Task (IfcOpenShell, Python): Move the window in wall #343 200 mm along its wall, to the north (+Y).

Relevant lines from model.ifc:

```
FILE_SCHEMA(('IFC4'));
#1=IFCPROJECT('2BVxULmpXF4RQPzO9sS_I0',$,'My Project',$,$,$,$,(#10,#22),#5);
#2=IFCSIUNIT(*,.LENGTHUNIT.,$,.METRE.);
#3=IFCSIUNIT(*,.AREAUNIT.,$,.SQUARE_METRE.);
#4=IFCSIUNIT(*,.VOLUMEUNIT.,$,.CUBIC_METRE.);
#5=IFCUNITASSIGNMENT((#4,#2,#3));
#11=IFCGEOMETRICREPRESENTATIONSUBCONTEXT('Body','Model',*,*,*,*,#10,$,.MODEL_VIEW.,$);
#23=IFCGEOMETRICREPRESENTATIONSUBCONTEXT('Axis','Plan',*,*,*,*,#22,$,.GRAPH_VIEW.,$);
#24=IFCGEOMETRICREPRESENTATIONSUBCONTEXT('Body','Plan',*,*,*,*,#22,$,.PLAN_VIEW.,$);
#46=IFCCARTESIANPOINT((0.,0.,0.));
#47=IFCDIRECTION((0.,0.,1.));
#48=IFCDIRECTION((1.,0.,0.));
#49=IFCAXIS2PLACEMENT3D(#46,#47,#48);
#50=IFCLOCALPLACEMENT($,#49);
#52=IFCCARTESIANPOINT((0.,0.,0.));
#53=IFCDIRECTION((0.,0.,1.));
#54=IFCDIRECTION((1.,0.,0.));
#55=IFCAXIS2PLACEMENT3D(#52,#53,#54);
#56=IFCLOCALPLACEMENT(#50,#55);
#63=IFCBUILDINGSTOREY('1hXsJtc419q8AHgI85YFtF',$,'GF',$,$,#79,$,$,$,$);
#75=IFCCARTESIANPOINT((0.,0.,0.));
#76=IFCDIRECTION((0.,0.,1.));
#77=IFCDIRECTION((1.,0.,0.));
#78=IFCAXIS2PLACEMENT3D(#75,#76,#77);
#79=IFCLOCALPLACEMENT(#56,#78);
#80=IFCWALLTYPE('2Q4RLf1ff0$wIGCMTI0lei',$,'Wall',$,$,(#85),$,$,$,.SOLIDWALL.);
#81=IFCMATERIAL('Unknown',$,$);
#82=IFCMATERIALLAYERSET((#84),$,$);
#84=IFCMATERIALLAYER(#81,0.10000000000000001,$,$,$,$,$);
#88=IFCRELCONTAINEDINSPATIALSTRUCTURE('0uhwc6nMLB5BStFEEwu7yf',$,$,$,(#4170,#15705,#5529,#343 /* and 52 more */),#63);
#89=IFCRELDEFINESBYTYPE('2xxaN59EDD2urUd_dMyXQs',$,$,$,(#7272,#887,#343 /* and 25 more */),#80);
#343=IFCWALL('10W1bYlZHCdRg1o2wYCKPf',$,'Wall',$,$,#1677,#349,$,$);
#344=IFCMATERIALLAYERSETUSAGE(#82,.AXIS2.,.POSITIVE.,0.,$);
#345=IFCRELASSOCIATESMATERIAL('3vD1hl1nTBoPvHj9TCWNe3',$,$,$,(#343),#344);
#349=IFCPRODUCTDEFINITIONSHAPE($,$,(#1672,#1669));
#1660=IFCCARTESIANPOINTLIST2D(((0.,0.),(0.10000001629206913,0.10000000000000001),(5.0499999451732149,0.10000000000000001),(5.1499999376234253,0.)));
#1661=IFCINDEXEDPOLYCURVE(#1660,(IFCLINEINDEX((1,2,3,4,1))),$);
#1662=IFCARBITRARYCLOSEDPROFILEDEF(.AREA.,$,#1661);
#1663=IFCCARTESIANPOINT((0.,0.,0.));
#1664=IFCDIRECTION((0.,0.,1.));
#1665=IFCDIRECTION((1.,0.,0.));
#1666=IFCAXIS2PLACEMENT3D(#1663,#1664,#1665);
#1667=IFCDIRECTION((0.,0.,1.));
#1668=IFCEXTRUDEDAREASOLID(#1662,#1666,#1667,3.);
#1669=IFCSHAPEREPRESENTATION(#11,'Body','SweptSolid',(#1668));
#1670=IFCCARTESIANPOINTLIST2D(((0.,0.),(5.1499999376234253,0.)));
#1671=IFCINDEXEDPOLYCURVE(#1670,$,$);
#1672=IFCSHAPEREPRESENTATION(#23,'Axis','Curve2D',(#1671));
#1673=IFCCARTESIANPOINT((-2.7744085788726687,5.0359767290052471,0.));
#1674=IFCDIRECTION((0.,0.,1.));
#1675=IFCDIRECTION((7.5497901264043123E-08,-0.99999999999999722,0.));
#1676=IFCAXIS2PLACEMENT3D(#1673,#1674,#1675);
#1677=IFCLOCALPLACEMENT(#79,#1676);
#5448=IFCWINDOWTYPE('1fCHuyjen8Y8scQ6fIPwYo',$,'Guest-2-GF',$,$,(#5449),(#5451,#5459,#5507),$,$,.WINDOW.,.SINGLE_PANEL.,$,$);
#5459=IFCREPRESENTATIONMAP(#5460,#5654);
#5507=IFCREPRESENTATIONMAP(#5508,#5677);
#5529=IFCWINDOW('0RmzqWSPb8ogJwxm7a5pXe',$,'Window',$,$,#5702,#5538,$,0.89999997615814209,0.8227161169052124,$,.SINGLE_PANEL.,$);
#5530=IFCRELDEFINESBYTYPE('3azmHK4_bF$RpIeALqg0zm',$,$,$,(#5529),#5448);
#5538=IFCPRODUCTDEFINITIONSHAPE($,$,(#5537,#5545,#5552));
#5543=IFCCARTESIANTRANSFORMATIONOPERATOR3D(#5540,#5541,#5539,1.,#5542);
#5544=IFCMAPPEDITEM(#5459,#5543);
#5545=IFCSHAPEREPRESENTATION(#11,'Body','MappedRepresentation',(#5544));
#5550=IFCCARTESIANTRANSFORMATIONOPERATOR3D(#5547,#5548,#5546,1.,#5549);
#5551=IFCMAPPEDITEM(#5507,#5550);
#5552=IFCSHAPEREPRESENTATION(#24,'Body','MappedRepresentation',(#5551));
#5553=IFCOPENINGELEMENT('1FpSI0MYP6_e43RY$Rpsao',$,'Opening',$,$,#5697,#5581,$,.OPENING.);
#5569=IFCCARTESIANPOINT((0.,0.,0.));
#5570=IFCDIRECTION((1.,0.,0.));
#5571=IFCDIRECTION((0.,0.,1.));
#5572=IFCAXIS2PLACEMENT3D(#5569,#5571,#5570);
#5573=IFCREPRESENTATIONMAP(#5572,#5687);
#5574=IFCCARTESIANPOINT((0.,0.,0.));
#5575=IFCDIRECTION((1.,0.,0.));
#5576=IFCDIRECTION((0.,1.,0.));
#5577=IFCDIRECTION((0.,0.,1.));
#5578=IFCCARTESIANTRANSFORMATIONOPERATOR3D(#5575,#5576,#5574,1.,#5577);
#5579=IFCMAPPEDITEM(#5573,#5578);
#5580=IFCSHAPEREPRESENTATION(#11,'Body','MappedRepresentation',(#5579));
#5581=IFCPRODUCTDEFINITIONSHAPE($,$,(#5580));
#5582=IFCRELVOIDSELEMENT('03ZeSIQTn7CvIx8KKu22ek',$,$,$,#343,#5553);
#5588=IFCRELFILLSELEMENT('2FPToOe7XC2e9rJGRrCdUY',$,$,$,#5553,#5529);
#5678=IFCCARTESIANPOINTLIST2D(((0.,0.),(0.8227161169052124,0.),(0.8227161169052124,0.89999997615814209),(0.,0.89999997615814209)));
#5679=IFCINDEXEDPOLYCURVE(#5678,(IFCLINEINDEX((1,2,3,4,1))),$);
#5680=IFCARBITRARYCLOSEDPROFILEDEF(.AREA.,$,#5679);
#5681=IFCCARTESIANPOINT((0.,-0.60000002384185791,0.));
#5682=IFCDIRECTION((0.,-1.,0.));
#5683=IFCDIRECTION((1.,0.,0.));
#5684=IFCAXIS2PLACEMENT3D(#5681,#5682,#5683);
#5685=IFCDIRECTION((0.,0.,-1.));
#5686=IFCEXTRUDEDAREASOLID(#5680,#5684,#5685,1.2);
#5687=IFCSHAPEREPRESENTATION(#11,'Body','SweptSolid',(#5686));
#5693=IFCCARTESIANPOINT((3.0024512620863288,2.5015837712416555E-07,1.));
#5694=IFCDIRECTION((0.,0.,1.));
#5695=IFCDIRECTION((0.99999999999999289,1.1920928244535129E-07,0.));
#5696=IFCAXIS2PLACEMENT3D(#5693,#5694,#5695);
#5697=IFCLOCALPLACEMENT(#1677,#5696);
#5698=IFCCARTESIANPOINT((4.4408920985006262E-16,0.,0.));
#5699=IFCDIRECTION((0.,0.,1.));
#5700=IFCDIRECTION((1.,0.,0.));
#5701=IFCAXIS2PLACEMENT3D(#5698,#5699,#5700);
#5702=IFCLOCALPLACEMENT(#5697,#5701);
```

```python
import ifcopenshell
import ifcopenshell.api.geometry
import ifcopenshell.util.placement
import ifcopenshell.util.unit

model = ifcopenshell.open("model.ifc")
unit_scale = ifcopenshell.util.unit.calculate_unit_scale(model)

window = model.by_id(5529)
opening = window.FillsVoids[0].RelatingOpeningElement
wall = opening.VoidsElements[0].RelatingBuildingElement

wall_matrix = ifcopenshell.util.placement.get_local_placement(wall.ObjectPlacement)
shift = wall_matrix[:3, 0] * -0.2 / unit_scale
before = ifcopenshell.util.placement.get_local_placement(window.ObjectPlacement)[:3, 3].copy()

# The window is placed relative to its opening, so it follows when the opening moves.
matrix = ifcopenshell.util.placement.get_local_placement(opening.ObjectPlacement)
matrix[:3, 3] += shift
ifcopenshell.api.geometry.edit_object_placement(
    model, product=opening, matrix=matrix, is_si=False, should_transform_children=True
)

after = ifcopenshell.util.placement.get_local_placement(window.ObjectPlacement)[:3, 3]
print("window moved by", (after - before).round(3) + 0.0)

model.write("model_rev.ifc")
```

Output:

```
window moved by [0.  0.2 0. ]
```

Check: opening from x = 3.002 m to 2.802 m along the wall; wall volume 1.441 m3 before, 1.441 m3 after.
